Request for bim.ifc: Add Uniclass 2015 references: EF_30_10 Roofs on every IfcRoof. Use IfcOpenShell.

First a look at what the model holds.

```python
import ifcopenshell

model = ifcopenshell.open("bim.ifc")
print(model.schema)
print("classifications:", [c.Name for c in model.by_type("IfcClassification")])
for ifc_class in ("IfcDoor", "IfcRoof", "IfcStair", "IfcWall", "IfcWindow"):
    print(ifc_class, len(model.by_type(ifc_class)))
```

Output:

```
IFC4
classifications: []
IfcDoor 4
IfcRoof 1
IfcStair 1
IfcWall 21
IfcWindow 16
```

```python
import ifcopenshell
import ifcopenshell.api.classification

model = ifcopenshell.open("bim.ifc")

system = ifcopenshell.api.classification.add_classification(model, classification="Uniclass 2015")

codes = {
    "IfcRoof": ("EF_30_10", "Roofs"),
}
for ifc_class, (code, name) in codes.items():
    products = model.by_type(ifc_class)
    ifcopenshell.api.classification.add_reference(
        model, products=products, classification=system, identification=code, name=name
    )
    print(code, len(products))

model.write("bim_edited.ifc")
```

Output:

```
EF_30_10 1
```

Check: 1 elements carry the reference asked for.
